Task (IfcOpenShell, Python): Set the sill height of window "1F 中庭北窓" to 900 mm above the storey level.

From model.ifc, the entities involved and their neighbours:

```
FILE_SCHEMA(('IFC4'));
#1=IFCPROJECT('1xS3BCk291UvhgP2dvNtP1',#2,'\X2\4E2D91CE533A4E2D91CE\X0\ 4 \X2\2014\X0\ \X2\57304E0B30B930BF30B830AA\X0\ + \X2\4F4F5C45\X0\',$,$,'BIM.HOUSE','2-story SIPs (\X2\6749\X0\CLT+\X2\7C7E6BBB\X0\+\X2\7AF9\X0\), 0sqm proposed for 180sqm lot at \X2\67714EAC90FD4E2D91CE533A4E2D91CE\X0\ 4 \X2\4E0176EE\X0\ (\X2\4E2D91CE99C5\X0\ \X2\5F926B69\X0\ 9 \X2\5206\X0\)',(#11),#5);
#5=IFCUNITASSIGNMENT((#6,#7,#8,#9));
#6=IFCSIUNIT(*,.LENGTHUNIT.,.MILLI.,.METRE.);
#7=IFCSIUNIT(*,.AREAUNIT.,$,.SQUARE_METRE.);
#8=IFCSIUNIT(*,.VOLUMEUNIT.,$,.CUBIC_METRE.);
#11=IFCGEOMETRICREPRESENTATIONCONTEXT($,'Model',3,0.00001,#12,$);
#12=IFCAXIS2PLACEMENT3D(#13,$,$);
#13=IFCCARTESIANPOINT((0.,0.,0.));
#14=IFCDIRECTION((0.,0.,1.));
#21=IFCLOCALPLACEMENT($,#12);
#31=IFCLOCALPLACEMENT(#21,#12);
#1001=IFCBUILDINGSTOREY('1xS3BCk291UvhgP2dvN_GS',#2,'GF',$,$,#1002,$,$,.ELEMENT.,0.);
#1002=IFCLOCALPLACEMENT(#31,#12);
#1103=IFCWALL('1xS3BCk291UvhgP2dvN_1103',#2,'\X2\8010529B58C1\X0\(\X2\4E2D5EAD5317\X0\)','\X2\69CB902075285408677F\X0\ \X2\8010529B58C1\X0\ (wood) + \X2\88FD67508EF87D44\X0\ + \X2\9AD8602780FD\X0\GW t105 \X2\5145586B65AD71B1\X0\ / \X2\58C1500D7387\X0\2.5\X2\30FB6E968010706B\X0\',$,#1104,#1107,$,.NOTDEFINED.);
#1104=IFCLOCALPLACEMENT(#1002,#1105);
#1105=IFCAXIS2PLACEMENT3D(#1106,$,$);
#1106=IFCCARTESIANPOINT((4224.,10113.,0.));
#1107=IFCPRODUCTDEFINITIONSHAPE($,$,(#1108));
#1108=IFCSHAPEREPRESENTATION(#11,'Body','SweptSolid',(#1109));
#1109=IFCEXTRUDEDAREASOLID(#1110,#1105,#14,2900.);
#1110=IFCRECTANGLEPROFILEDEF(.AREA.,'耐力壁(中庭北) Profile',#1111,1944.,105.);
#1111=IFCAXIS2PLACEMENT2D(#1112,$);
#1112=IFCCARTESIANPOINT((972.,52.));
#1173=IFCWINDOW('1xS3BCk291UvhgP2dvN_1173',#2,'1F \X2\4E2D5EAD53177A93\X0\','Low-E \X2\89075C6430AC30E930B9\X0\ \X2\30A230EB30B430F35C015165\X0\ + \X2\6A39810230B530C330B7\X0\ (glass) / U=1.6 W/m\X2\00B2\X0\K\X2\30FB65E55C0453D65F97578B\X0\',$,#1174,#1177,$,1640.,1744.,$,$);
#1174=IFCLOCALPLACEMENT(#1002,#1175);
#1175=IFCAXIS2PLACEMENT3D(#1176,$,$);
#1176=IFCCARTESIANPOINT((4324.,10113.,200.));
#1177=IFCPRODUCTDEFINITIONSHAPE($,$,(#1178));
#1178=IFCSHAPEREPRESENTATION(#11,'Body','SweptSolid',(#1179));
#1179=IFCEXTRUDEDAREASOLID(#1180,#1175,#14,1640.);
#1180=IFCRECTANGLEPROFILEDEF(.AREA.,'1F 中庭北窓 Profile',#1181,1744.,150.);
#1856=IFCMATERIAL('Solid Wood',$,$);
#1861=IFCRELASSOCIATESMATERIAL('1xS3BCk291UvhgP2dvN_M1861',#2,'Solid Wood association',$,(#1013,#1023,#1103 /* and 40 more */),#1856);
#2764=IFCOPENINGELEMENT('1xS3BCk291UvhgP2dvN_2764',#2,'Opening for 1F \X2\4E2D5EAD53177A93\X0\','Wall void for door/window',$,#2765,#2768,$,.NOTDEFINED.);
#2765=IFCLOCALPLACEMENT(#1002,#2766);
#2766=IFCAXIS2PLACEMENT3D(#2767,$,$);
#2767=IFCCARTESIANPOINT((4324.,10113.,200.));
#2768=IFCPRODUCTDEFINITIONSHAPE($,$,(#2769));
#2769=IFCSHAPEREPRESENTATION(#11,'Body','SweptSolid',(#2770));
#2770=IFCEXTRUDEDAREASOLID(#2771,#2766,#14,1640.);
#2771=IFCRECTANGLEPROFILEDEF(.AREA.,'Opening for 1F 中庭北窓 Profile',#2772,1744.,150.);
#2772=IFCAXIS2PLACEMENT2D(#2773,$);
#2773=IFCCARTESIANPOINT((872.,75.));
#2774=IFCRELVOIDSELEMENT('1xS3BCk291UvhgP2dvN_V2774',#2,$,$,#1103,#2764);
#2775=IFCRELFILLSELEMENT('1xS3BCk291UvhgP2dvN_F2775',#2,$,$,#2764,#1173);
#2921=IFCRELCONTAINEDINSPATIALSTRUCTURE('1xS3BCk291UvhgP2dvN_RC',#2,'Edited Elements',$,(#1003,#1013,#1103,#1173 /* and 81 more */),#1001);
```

```python
import numpy as np
import ifcopenshell
import ifcopenshell.api.geometry
import ifcopenshell.geom
import ifcopenshell.util.element
import ifcopenshell.util.placement
import ifcopenshell.util.shape
import ifcopenshell.util.unit

model = ifcopenshell.open("model.ifc")
unit_scale = ifcopenshell.util.unit.calculate_unit_scale(model)

window = model.by_guid("1xS3BCk291UvhgP2dvN_1173")
opening = window.FillsVoids[0].RelatingOpeningElement
storey = ifcopenshell.util.element.get_container(window, ifc_class="IfcBuildingStorey")
level = ifcopenshell.util.placement.get_local_placement(storey.ObjectPlacement)[2, 3]

# The opening's origin need not be at the sill, so measure its lowest point.
shape = ifcopenshell.geom.create_shape(ifcopenshell.geom.settings(), opening)
bottom = ifcopenshell.util.shape.get_shape_bottom_elevation(shape, shape.geometry) / unit_scale
dz = level + 900.0 - bottom

shift = np.array([0.0, 0.0, dz])
# The window is not placed relative to its opening, so move both.
for product in (opening, window):
    matrix = ifcopenshell.util.placement.get_local_placement(product.ObjectPlacement)
    matrix[:3, 3] += shift
    ifcopenshell.api.geometry.edit_object_placement(model, product=product, matrix=matrix, is_si=False)

print(f"moved by {dz * unit_scale:+.3f} m")

model.write("model-out.ifc")
```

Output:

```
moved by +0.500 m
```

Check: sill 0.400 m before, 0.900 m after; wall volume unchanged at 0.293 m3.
